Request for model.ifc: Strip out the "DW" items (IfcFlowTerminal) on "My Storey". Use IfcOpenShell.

First a look at what the model holds.

```python
import ifcopenshell
import ifcopenshell.util.element

model = ifcopenshell.open("model.ifc")
print(model.schema)
storey = next(s for s in model.by_type("IfcBuildingStorey") if s.Name == "My Storey")
terminals = [e for e in ifcopenshell.util.element.get_decomposition(storey) if e.is_a("IfcFlowTerminal")]
seen = {}
for e in terminals:
    element_type = ifcopenshell.util.element.get_type(e)
    name = element_type.Name if element_type not in (None, e) else None
    seen[name] = seen.get(name, 0) + 1
for name, count in sorted(seen.items(), key=str):
    print(count, "x", name)
```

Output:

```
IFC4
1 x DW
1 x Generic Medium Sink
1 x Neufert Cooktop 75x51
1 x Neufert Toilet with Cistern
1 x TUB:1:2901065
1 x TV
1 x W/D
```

```python
import ifcopenshell
import ifcopenshell.api.root
import ifcopenshell.util.element

model = ifcopenshell.open("model.ifc")

storey = next(s for s in model.by_type("IfcBuildingStorey") if s.Name == "My Storey")
terminals = [e for e in ifcopenshell.util.element.get_decomposition(storey) if e.is_a("IfcFlowTerminal")]
targets = [e for e in terminals if (t := ifcopenshell.util.element.get_type(e)) not in (None, e) and t.Name == "DW"]

for e in targets:
    ifcopenshell.api.root.remove_product(model, product=e)
print(len(targets), "removed")

model.write("model-out.ifc")
```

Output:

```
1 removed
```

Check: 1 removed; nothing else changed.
